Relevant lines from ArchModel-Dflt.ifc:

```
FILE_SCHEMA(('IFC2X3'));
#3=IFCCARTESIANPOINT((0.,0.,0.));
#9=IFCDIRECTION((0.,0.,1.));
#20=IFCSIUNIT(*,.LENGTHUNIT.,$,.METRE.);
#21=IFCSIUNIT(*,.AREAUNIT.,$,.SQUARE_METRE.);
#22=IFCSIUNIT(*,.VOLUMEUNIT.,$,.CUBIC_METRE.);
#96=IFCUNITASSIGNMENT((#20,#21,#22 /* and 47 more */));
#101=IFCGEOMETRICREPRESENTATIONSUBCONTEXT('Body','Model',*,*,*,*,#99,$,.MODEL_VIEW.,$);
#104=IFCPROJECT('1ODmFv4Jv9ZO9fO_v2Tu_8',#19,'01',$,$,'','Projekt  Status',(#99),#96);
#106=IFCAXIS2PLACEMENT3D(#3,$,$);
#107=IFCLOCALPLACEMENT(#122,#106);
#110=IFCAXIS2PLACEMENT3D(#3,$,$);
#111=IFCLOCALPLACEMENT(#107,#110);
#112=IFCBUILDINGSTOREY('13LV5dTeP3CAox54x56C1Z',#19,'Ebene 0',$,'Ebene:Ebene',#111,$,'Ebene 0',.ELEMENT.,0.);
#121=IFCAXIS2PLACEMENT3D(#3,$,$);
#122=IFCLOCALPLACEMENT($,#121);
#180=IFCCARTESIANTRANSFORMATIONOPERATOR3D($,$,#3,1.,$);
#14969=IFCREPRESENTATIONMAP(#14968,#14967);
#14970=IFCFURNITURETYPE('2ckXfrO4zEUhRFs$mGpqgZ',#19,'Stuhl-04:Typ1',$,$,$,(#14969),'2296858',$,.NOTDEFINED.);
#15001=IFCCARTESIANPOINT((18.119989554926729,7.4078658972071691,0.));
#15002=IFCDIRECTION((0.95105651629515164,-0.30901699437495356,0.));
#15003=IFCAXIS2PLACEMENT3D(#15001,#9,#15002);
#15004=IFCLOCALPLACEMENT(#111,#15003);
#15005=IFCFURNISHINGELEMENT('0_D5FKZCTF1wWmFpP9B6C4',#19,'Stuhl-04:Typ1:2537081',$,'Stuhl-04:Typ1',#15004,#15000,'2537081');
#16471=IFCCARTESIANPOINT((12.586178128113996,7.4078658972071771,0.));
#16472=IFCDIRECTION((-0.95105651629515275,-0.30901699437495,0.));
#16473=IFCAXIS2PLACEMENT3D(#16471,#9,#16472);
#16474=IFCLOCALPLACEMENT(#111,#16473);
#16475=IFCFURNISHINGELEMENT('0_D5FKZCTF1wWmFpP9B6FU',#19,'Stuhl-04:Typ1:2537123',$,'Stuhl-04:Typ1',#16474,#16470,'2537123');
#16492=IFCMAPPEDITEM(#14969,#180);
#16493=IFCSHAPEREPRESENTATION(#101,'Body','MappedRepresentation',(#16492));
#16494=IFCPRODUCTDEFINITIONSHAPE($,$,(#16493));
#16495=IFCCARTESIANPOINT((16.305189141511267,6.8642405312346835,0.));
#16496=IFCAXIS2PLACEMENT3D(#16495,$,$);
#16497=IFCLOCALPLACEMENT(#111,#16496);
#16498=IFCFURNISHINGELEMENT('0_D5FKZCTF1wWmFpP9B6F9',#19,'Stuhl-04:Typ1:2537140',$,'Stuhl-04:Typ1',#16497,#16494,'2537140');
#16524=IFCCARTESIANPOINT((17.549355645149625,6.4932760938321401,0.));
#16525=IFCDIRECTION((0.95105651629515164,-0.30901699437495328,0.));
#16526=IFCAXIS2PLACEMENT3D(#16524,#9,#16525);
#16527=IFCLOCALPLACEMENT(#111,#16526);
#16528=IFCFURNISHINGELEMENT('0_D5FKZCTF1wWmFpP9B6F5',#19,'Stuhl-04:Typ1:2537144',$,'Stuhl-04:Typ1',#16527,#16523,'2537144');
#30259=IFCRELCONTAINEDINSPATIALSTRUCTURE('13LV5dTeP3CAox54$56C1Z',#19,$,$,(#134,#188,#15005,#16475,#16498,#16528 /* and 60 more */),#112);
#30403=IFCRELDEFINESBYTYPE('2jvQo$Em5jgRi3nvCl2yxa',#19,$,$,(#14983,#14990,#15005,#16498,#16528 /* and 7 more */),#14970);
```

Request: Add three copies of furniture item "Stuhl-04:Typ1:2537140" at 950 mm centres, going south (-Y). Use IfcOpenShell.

```python
import numpy as np
import ifcopenshell
import ifcopenshell.api.geometry
import ifcopenshell.api.root
import ifcopenshell.util.element
import ifcopenshell.util.placement

model = ifcopenshell.open("ArchModel-Dflt.ifc")

source = model.by_id(16498)
base = ifcopenshell.util.placement.get_local_placement(source.ObjectPlacement)
step = np.array([0.0, -1.0, 0.0]) * 0.95

for i in range(1, 4):
    copy = ifcopenshell.api.root.copy_class(model, product=source)
    copy.Representation = ifcopenshell.util.element.copy_deep(
        model, source.Representation, exclude=["IfcGeometricRepresentationContext", "IfcRepresentationMap"]
    )
    copy.Name = "Stuhl-04:Typ1"
    copy.Tag = None
    matrix = base.copy()
    matrix[:3, 3] += i * step
    print("added at", matrix[:3, 3].round(3) + 0.0)
    ifcopenshell.api.geometry.edit_object_placement(model, product=copy, matrix=matrix, is_si=False)

model.write("ArchModel-Dflt_rev.ifc")
```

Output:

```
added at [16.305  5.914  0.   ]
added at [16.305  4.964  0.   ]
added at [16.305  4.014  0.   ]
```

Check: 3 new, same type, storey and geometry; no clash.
